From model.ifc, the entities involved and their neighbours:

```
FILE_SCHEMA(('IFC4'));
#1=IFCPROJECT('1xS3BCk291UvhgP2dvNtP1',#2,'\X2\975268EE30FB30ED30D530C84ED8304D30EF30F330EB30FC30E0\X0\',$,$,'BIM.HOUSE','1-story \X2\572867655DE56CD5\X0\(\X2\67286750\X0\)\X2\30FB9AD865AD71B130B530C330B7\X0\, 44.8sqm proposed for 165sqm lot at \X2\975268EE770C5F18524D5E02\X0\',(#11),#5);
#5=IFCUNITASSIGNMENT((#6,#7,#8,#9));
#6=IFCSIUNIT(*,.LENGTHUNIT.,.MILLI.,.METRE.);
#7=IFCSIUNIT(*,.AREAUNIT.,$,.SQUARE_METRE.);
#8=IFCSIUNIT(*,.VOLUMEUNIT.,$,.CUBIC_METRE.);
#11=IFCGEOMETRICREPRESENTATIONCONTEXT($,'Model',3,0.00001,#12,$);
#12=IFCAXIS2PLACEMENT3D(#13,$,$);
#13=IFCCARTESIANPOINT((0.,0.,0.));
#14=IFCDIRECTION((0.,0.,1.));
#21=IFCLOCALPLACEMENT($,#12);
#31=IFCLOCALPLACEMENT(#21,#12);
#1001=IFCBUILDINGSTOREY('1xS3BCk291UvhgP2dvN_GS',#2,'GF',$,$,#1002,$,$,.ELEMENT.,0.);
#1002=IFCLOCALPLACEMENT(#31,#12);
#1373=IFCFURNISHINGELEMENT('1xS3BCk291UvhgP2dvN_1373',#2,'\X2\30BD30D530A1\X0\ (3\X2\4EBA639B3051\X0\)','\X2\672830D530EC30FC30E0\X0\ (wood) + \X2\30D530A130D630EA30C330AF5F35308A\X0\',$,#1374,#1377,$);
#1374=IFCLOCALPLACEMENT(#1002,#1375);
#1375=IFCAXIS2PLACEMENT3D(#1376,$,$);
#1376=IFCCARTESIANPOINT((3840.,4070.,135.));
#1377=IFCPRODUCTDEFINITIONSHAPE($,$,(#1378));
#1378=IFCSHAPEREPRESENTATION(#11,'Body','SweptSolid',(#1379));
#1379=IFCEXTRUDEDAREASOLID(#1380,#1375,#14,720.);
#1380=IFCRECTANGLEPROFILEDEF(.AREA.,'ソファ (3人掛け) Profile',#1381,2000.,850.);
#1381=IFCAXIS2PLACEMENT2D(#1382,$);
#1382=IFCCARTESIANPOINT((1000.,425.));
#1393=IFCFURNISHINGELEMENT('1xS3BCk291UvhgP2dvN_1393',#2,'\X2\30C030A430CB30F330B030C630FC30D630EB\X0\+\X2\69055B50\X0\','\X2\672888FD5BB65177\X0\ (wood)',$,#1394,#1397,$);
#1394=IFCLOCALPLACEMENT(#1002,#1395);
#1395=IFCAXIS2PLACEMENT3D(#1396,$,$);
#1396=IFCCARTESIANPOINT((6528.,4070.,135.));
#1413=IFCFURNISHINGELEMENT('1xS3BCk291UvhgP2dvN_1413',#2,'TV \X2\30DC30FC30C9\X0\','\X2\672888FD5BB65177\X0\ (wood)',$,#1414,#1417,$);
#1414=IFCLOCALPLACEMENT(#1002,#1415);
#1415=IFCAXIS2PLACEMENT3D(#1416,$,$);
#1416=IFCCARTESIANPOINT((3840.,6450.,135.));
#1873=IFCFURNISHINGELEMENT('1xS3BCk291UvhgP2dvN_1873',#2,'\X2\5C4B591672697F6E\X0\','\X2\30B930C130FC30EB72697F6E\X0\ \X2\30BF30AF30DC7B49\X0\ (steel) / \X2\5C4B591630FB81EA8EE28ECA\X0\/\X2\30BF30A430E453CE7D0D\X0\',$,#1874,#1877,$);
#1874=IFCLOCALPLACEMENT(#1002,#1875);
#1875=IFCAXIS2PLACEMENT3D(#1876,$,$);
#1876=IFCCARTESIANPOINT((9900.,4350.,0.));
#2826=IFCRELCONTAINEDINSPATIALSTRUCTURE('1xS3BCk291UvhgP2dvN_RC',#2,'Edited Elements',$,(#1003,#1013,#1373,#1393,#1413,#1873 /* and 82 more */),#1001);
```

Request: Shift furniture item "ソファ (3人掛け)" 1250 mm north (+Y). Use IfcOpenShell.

```python
import ifcopenshell
import ifcopenshell.api.geometry
import ifcopenshell.util.placement
import ifcopenshell.util.unit

model = ifcopenshell.open("model.ifc")
unit_scale = ifcopenshell.util.unit.calculate_unit_scale(model)

item = model.by_guid("1xS3BCk291UvhgP2dvN_1373")
matrix = ifcopenshell.util.placement.get_local_placement(item.ObjectPlacement)
matrix[1, 3] += 1.25 / unit_scale
ifcopenshell.api.geometry.edit_object_placement(model, product=item, matrix=matrix, is_si=False)

print(ifcopenshell.util.placement.get_local_placement(item.ObjectPlacement).round(3) + 0.0)

model.write("model_v2.ifc")
```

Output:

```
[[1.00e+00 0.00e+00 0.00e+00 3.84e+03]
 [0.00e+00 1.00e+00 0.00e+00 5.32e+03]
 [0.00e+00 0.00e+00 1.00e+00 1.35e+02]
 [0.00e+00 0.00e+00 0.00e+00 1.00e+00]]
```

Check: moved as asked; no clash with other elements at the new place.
